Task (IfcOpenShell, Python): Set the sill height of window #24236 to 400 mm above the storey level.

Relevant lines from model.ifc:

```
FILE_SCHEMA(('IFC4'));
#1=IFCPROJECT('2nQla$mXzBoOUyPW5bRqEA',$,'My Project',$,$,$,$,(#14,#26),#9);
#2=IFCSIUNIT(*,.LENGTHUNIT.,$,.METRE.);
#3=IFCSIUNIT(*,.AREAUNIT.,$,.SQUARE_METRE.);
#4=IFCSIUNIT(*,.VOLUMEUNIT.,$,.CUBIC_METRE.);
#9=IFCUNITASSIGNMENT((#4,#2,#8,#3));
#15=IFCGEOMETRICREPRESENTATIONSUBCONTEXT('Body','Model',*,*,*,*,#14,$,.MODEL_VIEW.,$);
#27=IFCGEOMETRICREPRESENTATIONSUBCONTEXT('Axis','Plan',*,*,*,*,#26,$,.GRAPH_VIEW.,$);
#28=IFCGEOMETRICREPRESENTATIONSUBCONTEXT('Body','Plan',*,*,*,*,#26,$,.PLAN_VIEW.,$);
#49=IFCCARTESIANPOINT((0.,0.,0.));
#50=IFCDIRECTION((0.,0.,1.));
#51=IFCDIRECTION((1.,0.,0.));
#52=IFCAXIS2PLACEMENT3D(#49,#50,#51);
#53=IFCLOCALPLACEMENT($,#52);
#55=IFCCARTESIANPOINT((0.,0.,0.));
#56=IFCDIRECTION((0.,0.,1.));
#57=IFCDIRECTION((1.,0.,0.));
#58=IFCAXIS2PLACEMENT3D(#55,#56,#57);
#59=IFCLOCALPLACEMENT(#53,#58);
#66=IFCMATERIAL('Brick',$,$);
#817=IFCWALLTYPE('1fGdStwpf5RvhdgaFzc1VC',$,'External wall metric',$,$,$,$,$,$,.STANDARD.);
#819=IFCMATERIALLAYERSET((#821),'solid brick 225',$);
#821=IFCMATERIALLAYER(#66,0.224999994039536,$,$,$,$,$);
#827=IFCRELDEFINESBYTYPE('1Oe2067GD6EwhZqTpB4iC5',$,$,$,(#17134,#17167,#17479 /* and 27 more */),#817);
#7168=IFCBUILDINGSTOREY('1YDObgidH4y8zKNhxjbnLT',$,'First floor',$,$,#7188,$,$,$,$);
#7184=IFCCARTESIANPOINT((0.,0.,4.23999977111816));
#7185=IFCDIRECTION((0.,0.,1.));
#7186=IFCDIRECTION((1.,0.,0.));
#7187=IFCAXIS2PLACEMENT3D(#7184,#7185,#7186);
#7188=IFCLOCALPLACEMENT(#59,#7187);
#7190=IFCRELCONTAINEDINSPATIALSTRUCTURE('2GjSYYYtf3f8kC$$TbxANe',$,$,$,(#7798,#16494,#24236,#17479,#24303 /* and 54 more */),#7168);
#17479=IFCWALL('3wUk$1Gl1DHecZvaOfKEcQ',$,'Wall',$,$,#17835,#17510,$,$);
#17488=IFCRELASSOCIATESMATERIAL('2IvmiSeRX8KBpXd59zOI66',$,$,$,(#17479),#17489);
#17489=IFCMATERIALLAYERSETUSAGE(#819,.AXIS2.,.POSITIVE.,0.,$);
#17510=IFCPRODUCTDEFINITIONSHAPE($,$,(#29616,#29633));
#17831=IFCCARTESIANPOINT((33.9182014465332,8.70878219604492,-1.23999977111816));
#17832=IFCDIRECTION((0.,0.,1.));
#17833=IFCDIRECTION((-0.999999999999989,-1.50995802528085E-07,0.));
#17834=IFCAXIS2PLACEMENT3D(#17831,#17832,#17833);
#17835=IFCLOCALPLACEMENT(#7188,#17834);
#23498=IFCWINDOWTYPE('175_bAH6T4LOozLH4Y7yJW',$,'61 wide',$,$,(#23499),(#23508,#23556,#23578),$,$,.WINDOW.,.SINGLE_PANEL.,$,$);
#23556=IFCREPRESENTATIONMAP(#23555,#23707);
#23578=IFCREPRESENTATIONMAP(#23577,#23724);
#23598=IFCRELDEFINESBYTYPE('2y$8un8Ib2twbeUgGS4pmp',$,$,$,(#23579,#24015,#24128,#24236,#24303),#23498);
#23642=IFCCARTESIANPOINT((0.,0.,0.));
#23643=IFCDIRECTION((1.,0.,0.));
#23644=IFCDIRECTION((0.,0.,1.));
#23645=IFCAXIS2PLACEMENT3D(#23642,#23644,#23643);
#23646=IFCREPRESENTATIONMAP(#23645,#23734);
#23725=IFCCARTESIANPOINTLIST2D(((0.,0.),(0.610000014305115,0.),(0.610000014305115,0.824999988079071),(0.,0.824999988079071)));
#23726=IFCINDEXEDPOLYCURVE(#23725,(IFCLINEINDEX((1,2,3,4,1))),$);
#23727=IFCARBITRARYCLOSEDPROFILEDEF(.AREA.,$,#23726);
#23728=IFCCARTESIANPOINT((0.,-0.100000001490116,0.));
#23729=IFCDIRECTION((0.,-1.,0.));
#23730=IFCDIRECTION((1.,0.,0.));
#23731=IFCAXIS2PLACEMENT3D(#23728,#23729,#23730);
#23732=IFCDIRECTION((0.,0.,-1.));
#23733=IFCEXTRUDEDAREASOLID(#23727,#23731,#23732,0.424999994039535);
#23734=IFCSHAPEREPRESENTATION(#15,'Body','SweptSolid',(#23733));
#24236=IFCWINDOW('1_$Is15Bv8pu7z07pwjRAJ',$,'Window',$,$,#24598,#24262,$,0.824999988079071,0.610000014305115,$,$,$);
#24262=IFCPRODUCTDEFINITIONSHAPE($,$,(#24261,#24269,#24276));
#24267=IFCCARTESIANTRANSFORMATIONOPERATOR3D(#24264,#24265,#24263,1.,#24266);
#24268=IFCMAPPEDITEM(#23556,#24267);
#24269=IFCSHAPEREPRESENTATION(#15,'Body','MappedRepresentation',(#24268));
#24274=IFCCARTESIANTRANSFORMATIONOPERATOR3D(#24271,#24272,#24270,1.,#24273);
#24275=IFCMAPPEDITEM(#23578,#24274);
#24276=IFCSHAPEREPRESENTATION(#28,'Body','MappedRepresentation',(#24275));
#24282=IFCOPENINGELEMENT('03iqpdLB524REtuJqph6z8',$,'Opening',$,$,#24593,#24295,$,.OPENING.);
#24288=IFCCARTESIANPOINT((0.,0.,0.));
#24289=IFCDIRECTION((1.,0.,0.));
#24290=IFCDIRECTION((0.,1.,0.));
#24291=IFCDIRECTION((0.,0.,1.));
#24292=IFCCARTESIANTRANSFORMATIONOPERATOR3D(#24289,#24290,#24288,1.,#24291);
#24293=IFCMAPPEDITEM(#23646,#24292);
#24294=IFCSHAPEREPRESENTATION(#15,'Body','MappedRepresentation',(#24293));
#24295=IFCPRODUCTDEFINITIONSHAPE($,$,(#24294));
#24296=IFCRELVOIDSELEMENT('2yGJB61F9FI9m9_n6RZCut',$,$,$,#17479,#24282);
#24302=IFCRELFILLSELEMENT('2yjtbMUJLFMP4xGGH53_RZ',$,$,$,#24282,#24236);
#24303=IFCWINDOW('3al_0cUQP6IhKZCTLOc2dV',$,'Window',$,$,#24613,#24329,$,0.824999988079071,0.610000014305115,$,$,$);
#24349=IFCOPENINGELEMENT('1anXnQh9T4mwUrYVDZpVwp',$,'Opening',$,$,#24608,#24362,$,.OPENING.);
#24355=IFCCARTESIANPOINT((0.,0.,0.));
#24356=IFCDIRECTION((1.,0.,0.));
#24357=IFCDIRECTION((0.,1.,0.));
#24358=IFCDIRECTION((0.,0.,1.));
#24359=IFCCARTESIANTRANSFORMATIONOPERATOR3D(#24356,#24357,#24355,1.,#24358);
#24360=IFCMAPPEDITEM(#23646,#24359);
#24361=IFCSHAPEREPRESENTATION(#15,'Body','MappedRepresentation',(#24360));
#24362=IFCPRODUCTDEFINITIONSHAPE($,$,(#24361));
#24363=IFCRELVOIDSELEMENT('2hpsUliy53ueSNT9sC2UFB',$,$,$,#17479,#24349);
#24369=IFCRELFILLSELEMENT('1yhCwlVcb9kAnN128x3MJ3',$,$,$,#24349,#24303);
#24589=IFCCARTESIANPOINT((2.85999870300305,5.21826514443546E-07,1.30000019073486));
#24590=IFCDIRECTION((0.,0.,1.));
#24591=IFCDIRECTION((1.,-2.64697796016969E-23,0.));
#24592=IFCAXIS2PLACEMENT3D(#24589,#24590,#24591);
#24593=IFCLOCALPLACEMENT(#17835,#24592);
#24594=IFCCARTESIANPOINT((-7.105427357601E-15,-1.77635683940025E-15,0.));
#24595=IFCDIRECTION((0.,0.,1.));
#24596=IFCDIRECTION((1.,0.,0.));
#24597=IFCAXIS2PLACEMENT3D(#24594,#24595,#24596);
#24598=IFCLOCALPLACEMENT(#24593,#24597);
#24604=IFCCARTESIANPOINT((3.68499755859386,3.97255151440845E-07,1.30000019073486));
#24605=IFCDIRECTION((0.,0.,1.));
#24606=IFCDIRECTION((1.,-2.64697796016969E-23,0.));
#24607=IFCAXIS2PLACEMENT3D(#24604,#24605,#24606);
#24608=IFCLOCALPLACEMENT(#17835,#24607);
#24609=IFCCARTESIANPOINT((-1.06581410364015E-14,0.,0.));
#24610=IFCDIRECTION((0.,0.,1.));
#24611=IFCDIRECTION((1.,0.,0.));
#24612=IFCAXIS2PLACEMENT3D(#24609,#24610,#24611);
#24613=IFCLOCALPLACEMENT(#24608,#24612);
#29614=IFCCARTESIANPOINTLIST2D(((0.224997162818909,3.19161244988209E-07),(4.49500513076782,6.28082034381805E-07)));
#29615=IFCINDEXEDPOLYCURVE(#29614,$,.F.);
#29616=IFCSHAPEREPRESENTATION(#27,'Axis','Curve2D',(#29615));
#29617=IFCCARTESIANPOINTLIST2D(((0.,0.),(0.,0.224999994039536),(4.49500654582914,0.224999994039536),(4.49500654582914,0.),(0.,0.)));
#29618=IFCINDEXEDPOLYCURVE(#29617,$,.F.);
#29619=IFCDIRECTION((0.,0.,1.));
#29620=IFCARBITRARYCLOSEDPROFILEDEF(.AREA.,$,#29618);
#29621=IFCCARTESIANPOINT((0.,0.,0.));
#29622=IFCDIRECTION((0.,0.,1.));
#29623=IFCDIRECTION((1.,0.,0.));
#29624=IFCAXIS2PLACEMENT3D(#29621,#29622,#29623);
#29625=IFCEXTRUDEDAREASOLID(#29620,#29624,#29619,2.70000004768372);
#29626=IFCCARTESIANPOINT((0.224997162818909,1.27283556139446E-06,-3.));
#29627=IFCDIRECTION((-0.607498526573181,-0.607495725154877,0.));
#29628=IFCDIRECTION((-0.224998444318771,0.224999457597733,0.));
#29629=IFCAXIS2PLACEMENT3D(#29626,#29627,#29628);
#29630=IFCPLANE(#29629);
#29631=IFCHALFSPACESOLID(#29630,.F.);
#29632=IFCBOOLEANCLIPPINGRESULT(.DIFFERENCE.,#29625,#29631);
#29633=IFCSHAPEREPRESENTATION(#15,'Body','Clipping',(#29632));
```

```python
import numpy as np
import ifcopenshell
import ifcopenshell.api.geometry
import ifcopenshell.geom
import ifcopenshell.util.element
import ifcopenshell.util.placement
import ifcopenshell.util.shape
import ifcopenshell.util.unit

model = ifcopenshell.open("model.ifc")
unit_scale = ifcopenshell.util.unit.calculate_unit_scale(model)

window = model.by_guid("1_$Is15Bv8pu7z07pwjRAJ")
opening = window.FillsVoids[0].RelatingOpeningElement
storey = ifcopenshell.util.element.get_container(window, ifc_class="IfcBuildingStorey")
level = ifcopenshell.util.placement.get_local_placement(storey.ObjectPlacement)[2, 3]

# The opening's origin need not be at the sill, so measure its lowest point.
shape = ifcopenshell.geom.create_shape(ifcopenshell.geom.settings(), opening)
bottom = ifcopenshell.util.shape.get_shape_bottom_elevation(shape, shape.geometry) / unit_scale
dz = level + 0.4 - bottom

shift = np.array([0.0, 0.0, dz])
# The window is placed relative to its opening, so it follows when the opening moves.
matrix = ifcopenshell.util.placement.get_local_placement(opening.ObjectPlacement)
matrix[:3, 3] += shift
ifcopenshell.api.geometry.edit_object_placement(
    model, product=opening, matrix=matrix, is_si=False, should_transform_children=True
)

print(f"moved by {dz * unit_scale:+.3f} m")

model.write("model_edited.ifc")
```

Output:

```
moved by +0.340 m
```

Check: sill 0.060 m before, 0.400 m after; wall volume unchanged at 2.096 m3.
